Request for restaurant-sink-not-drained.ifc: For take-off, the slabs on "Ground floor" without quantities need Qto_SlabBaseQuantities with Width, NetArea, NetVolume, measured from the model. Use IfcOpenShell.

First a look at what the model holds.

```python
import ifcopenshell
import ifcopenshell.util.element
import ifcopenshell.util.unit

model = ifcopenshell.open("restaurant-sink-not-drained.ifc")
print(model.schema)
for unit_type in ("LENGTHUNIT", "AREAUNIT", "VOLUMEUNIT"):
    print(unit_type, ifcopenshell.util.unit.calculate_unit_scale(model, unit_type))
storey = next(s for s in model.by_type("IfcBuildingStorey") if s.Name == "Ground floor")
slabs = [e for e in ifcopenshell.util.element.get_decomposition(storey) if e.is_a("IfcSlab")]
for e in sorted(slabs, key=lambda e: e.id()):
    print(e.id(), e.is_a(), e.Name, list(ifcopenshell.util.element.get_psets(e, qtos_only=True)), sep=" | ")
```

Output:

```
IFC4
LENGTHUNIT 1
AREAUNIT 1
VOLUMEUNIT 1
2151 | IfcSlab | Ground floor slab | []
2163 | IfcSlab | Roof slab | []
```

```python
import ifcopenshell
import ifcopenshell.api.pset
import ifcopenshell.geom
import ifcopenshell.util.element
import ifcopenshell.util.shape
import ifcopenshell.util.unit

model = ifcopenshell.open("restaurant-sink-not-drained.ifc")
unit_scale = ifcopenshell.util.unit.calculate_unit_scale(model)
area_scale = ifcopenshell.util.unit.calculate_unit_scale(model, "AREAUNIT")
volume_scale = ifcopenshell.util.unit.calculate_unit_scale(model, "VOLUMEUNIT")
settings = ifcopenshell.geom.settings()

storey = next(s for s in model.by_type("IfcBuildingStorey") if s.Name == "Ground floor")
slabs = [e for e in ifcopenshell.util.element.get_decomposition(storey) if e.is_a("IfcSlab")]

for e in sorted(slabs, key=lambda e: e.id()):
    if ifcopenshell.util.element.get_psets(e, qtos_only=True, should_inherit=False):
        continue
    # Geometry comes back in metres, in the element's own axes.
    shape = ifcopenshell.geom.create_shape(settings, e)
    values = {
        "Width": ifcopenshell.util.shape.get_z(shape.geometry) / unit_scale,
        "NetArea": ifcopenshell.util.shape.get_footprint_area(shape.geometry) / area_scale,
        "NetVolume": ifcopenshell.util.shape.get_volume(shape.geometry) / volume_scale,
    }
    qto = ifcopenshell.api.pset.add_qto(model, product=e, name="Qto_SlabBaseQuantities")
    ifcopenshell.api.pset.edit_qto(model, qto=qto, properties=values)
    print(e.id(), {k: round(v, 3) for k, v in values.items()})

model.write("restaurant-sink-not-drained_rev.ifc")
```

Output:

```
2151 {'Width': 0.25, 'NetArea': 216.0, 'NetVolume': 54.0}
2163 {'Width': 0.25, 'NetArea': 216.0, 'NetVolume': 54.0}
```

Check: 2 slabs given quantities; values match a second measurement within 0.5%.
